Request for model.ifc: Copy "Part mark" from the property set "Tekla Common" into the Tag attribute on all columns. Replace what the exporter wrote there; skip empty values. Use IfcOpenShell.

First a look at what the model holds.

```python
import ifcopenshell
import ifcopenshell.util.element

model = ifcopenshell.open("model.ifc")
print(model.schema)
columns = model.by_type("IfcColumn")
print(len(columns), "columns")
for e in columns[:8]:
    source = ifcopenshell.util.element.get_pset(e, "Tekla Common", "Part mark")
    target = e.Tag
    print(e.id(), repr(source), repr(target), sep=" | ")
```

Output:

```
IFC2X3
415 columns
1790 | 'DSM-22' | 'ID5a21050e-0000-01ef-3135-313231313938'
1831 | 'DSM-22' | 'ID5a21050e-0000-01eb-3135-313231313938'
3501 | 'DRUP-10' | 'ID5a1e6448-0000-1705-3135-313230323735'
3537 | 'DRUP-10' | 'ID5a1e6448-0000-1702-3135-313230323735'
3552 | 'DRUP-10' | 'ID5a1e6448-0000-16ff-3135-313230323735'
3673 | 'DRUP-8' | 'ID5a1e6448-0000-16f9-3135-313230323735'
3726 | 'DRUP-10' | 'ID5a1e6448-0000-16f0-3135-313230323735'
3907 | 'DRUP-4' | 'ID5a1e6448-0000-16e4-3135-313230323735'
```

```python
import ifcopenshell
import ifcopenshell.util.element

model = ifcopenshell.open("model.ifc")

count = 0
for e in model.by_type("IfcColumn"):
    value = ifcopenshell.util.element.get_pset(e, "Tekla Common", "Part mark")
    current = e.Tag
    if not value or not value.strip() or current == value:
        continue
    e.Tag = value
    count += 1

print(count, "columns updated")

model.write("model_v2.ifc")
```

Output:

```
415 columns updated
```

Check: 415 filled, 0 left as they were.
